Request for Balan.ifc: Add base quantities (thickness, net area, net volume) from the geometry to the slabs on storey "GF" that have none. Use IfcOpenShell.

First a look at what the model holds.

```python
import ifcopenshell
import ifcopenshell.util.element
import ifcopenshell.util.unit

model = ifcopenshell.open("Balan.ifc")
print(model.schema)
for unit_type in ("LENGTHUNIT", "AREAUNIT", "VOLUMEUNIT"):
    print(unit_type, ifcopenshell.util.unit.calculate_unit_scale(model, unit_type))
storey = next(s for s in model.by_type("IfcBuildingStorey") if s.Name == "GF")
slabs = [e for e in ifcopenshell.util.element.get_decomposition(storey) if e.is_a("IfcSlab")]
for e in sorted(slabs, key=lambda e: e.id()):
    print(e.id(), e.is_a(), e.Name, list(ifcopenshell.util.element.get_psets(e, qtos_only=True)), sep=" | ")
```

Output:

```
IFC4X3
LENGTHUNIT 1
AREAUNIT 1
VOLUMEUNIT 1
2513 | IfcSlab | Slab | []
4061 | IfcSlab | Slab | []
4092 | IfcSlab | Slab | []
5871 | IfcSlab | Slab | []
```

```python
import ifcopenshell
import ifcopenshell.api.pset
import ifcopenshell.geom
import ifcopenshell.util.element
import ifcopenshell.util.shape
import ifcopenshell.util.unit

model = ifcopenshell.open("Balan.ifc")
unit_scale = ifcopenshell.util.unit.calculate_unit_scale(model)
area_scale = ifcopenshell.util.unit.calculate_unit_scale(model, "AREAUNIT")
volume_scale = ifcopenshell.util.unit.calculate_unit_scale(model, "VOLUMEUNIT")
settings = ifcopenshell.geom.settings()

storey = next(s for s in model.by_type("IfcBuildingStorey") if s.Name == "GF")
slabs = [e for e in ifcopenshell.util.element.get_decomposition(storey) if e.is_a("IfcSlab")]

for e in sorted(slabs, key=lambda e: e.id()):
    if ifcopenshell.util.element.get_psets(e, qtos_only=True, should_inherit=False):
        continue
    # Geometry comes back in metres, in the element's own axes.
    shape = ifcopenshell.geom.create_shape(settings, e)
    values = {
        "Width": ifcopenshell.util.shape.get_z(shape.geometry) / unit_scale,
        "NetArea": ifcopenshell.util.shape.get_footprint_area(shape.geometry) / area_scale,
        "NetVolume": ifcopenshell.util.shape.get_volume(shape.geometry) / volume_scale,
    }
    qto = ifcopenshell.api.pset.add_qto(model, product=e, name="Qto_SlabBaseQuantities")
    ifcopenshell.api.pset.edit_qto(model, qto=qto, properties=values)
    print(e.id(), {k: round(v, 3) for k, v in values.items()})

model.write("Balan_v2.ifc")
```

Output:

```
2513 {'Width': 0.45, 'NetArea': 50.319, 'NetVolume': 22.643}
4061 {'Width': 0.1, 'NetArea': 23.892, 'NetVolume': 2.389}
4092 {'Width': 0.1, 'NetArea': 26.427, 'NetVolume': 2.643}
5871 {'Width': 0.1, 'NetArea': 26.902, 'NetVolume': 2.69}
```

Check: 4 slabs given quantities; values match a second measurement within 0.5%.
